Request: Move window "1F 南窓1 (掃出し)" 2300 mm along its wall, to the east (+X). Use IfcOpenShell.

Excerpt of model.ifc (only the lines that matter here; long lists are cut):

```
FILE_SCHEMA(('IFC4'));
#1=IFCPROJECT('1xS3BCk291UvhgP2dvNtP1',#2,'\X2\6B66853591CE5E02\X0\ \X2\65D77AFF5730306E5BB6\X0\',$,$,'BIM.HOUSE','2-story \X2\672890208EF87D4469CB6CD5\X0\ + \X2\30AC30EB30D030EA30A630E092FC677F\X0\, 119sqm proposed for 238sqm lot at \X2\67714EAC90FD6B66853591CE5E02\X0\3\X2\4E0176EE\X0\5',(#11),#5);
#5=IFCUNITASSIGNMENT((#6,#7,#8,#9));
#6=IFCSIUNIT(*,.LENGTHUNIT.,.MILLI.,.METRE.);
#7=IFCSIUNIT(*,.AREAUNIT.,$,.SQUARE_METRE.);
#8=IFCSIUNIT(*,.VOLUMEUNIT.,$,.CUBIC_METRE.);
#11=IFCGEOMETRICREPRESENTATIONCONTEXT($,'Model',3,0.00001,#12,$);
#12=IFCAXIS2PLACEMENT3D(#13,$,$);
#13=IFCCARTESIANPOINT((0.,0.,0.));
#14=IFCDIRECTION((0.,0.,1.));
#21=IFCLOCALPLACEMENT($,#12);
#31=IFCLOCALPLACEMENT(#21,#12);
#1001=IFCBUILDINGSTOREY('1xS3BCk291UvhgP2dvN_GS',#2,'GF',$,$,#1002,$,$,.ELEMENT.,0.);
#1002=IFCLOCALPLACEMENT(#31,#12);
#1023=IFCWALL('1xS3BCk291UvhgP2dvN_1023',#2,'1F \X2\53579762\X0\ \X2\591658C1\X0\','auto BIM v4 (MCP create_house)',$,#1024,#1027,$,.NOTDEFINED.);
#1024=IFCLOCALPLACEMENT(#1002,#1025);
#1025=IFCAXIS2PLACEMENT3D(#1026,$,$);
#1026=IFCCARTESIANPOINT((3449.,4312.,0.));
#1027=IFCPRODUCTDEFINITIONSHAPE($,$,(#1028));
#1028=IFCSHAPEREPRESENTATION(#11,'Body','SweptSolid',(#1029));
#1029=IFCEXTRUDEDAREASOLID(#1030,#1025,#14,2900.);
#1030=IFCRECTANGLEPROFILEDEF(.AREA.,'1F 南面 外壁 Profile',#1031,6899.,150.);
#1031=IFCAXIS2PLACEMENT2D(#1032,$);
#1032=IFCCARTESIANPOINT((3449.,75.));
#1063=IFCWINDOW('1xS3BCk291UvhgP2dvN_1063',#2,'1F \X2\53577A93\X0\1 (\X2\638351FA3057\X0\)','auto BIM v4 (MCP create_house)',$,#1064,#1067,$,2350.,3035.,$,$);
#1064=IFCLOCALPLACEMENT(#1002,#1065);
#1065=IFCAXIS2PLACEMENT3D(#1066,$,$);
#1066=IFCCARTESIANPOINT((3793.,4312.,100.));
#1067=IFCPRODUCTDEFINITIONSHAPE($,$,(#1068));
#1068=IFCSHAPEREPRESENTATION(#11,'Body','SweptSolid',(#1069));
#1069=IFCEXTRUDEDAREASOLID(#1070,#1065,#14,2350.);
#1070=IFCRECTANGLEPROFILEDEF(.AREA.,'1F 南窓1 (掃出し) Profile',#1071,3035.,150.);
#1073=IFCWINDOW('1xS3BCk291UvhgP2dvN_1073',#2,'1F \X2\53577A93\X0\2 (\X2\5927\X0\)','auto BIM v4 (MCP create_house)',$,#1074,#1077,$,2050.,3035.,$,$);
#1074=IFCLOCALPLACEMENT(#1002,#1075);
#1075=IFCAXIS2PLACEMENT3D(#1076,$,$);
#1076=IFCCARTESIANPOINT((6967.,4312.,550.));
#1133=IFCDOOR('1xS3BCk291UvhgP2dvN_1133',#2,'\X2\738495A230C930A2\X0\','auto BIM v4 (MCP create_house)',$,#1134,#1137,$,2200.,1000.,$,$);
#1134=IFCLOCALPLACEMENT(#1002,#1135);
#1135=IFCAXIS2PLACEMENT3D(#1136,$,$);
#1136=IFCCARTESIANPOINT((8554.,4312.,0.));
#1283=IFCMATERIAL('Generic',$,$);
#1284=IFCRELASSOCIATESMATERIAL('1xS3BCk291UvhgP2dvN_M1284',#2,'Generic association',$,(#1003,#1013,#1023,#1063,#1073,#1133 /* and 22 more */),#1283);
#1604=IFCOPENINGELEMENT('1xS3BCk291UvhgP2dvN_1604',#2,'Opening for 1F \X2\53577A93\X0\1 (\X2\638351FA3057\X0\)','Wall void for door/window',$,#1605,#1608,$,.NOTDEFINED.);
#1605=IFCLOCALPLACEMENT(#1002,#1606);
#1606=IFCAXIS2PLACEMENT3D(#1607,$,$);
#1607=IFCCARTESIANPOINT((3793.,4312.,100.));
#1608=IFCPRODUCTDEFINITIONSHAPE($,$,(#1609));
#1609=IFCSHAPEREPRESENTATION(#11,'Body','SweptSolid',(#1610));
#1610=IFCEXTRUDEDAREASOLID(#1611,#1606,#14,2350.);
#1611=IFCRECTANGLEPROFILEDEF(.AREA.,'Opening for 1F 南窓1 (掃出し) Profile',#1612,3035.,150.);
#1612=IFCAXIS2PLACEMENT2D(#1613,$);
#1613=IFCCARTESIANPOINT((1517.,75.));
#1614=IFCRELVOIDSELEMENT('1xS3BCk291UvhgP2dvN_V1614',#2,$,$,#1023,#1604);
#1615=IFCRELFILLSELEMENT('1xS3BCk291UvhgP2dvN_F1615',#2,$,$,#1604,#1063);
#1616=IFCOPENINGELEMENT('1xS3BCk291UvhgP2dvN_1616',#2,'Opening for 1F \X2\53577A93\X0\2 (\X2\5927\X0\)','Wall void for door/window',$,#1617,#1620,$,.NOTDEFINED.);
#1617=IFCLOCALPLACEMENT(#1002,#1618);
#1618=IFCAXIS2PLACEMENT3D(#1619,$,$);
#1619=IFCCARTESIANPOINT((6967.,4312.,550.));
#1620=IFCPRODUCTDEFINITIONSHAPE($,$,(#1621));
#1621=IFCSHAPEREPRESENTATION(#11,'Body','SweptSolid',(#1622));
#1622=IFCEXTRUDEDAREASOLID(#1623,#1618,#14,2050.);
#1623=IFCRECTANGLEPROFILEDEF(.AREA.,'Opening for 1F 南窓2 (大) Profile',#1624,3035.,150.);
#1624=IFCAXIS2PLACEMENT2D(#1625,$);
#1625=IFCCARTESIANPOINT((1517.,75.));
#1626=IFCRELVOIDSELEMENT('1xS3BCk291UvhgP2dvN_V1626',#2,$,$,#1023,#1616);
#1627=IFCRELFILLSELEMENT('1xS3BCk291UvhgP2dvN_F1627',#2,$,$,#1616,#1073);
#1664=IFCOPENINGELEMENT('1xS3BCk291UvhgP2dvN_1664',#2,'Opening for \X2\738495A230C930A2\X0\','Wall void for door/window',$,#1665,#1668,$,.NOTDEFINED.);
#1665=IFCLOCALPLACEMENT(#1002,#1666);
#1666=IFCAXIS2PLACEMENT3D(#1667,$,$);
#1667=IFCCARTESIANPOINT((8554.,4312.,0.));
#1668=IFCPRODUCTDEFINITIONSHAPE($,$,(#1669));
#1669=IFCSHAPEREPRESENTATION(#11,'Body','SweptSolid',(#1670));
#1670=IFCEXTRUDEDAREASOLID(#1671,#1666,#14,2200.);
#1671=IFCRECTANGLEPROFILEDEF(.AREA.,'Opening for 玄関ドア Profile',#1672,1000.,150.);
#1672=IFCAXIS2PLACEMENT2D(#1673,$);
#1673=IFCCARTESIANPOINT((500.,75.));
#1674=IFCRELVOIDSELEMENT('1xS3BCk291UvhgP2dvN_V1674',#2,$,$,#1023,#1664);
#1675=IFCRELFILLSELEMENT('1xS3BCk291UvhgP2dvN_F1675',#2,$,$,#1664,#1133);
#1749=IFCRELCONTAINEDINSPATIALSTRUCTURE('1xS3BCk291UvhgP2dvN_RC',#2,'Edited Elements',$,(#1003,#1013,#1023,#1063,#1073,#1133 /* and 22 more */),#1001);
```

```python
import ifcopenshell
import ifcopenshell.api.geometry
import ifcopenshell.util.placement

model = ifcopenshell.open("model.ifc")

window = model.by_guid("1xS3BCk291UvhgP2dvN_1063")
opening = window.FillsVoids[0].RelatingOpeningElement
wall = opening.VoidsElements[0].RelatingBuildingElement

wall_matrix = ifcopenshell.util.placement.get_local_placement(wall.ObjectPlacement)
shift = wall_matrix[:3, 0] * 2300.0
before = ifcopenshell.util.placement.get_local_placement(window.ObjectPlacement)[:3, 3].copy()

# The window is not placed relative to its opening, so move both.
for product in (opening, window):
    matrix = ifcopenshell.util.placement.get_local_placement(product.ObjectPlacement)
    matrix[:3, 3] += shift
    ifcopenshell.api.geometry.edit_object_placement(model, product=product, matrix=matrix, is_si=False)

after = ifcopenshell.util.placement.get_local_placement(window.ObjectPlacement)[:3, 3]
print("window moved by", (after - before).round(3) + 0.0)

model.write("model_rev.ifc")
```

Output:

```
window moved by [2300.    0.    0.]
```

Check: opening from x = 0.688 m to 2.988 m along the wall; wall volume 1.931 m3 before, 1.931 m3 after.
